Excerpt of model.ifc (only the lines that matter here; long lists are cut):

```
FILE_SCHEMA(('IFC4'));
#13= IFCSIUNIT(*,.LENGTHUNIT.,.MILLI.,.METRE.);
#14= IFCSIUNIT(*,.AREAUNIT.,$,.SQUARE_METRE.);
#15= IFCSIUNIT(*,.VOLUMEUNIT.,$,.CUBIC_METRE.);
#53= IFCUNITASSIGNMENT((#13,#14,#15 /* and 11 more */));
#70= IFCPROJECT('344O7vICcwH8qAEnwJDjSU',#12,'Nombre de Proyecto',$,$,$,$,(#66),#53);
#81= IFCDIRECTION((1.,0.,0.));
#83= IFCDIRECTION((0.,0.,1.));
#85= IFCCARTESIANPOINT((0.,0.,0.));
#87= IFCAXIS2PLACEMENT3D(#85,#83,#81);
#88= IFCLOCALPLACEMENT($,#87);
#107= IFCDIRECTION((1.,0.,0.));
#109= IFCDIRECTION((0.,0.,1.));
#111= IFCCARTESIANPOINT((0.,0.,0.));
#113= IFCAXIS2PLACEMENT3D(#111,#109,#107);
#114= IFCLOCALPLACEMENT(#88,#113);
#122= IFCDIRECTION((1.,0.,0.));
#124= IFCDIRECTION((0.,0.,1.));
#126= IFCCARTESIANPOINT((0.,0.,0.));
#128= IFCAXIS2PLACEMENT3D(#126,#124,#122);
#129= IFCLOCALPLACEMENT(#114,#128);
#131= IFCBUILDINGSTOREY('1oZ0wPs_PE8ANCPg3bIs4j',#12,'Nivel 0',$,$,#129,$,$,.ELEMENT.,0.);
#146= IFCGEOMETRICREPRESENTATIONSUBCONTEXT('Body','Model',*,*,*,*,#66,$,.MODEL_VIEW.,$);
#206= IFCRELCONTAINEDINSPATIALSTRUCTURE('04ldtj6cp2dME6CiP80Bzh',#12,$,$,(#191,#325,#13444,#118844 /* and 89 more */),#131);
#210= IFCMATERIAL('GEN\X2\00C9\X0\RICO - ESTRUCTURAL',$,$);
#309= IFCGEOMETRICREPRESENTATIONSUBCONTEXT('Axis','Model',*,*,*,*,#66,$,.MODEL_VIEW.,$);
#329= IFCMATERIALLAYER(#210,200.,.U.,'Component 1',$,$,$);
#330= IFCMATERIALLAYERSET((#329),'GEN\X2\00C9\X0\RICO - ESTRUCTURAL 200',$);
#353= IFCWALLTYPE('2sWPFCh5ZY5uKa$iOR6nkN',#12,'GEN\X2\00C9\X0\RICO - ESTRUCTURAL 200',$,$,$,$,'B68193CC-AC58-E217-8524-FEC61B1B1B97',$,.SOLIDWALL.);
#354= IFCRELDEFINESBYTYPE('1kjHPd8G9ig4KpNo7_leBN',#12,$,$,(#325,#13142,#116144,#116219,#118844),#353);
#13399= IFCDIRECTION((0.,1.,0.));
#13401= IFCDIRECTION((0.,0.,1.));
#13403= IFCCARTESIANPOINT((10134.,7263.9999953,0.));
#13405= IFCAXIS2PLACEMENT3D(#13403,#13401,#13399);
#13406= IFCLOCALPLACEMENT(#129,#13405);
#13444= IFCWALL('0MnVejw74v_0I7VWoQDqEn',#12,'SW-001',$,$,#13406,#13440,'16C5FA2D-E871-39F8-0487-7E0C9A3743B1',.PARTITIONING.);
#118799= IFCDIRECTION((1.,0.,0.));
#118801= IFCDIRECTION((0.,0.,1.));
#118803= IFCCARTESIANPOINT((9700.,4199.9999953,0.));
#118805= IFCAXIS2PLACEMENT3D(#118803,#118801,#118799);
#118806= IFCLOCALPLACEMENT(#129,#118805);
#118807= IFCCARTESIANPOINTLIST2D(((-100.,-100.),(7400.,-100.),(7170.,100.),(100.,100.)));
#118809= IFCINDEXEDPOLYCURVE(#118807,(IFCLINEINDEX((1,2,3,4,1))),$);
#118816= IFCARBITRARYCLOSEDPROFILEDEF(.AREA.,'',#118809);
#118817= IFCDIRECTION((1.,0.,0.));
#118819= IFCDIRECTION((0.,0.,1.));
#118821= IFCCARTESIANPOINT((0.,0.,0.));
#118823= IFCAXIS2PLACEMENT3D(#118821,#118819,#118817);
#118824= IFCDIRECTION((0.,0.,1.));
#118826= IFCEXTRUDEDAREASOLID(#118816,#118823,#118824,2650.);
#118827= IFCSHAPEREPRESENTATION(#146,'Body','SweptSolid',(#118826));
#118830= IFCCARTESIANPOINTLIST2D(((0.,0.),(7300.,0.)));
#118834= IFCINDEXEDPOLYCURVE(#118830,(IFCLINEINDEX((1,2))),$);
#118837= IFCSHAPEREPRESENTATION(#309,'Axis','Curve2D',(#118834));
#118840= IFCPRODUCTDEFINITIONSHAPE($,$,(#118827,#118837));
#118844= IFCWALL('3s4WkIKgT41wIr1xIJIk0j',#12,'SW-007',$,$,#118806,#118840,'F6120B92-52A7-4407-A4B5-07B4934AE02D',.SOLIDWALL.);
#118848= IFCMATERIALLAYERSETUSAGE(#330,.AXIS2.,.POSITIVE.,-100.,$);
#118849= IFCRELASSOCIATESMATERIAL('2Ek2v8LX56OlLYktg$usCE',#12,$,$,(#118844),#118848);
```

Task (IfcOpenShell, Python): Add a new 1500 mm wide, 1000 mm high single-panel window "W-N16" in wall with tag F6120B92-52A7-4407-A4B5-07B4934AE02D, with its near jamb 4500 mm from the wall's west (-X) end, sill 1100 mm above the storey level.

```python
import numpy as np
import ifcopenshell
import ifcopenshell.api.feature
import ifcopenshell.api.geometry
import ifcopenshell.api.root
import ifcopenshell.api.spatial
import ifcopenshell.geom
import ifcopenshell.util.element
import ifcopenshell.util.placement
import ifcopenshell.util.representation
import ifcopenshell.util.shape
import ifcopenshell.util.unit

model = ifcopenshell.open("model.ifc")
unit_scale = ifcopenshell.util.unit.calculate_unit_scale(model)
settings = ifcopenshell.geom.settings()


def volume(element):
    """Net volume in cubic metres, openings subtracted."""
    shape = ifcopenshell.geom.create_shape(settings, element)
    return ifcopenshell.util.shape.get_volume(shape.geometry)


wall = model.by_guid("3s4WkIKgT41wIr1xIJIk0j")
storey = ifcopenshell.util.element.get_container(wall, ifc_class="IfcBuildingStorey")
context = ifcopenshell.util.representation.get_context(model, "Model", "Body", "MODEL_VIEW")
before = volume(wall)

width, height, from_end, sill = 1.5, 1, 4.5, 1.1  # metres

# The wall runs along its own X axis, and the end named is its -X end.
wall_shape = ifcopenshell.geom.create_shape(settings, wall)
x, y, z = ifcopenshell.util.shape.get_vertices(wall_shape.geometry).T
start = x.min() + from_end
face, thickness = float(y.min()), float(y.max() - y.min())
wall_matrix = ifcopenshell.util.placement.get_local_placement(wall.ObjectPlacement)
level = ifcopenshell.util.placement.get_local_placement(storey.ObjectPlacement)[2, 3]


def in_wall(x, y):
    """Placement at x, y metres in the wall's axes, at sill height."""
    matrix = wall_matrix.copy()
    matrix[:, 3] = wall_matrix @ np.array([x / unit_scale, y / unit_scale, 0.0, 1.0])
    matrix[2, 3] = level + sill / unit_scale
    return matrix


# Opening: a box that overshoots both wall faces by 50 mm.
opening = ifcopenshell.api.root.create_entity(model, ifc_class="IfcOpeningElement", predefined_type="OPENING")
box = ifcopenshell.api.geometry.add_wall_representation(
    model, context=context, length=width, height=height, thickness=thickness + 0.1
)
ifcopenshell.api.geometry.assign_representation(model, product=opening, representation=box)
ifcopenshell.api.geometry.edit_object_placement(model, product=opening, matrix=in_wall(start, face - 0.05), is_si=False)
ifcopenshell.api.feature.add_feature(model, feature=opening, element=wall)

window = ifcopenshell.api.root.create_entity(model, ifc_class="IfcWindow", name="W-N16", predefined_type="WINDOW")
window.OverallWidth, window.OverallHeight = width / unit_scale, height / unit_scale
window.PartitioningType = "SINGLE_PANEL"
body = ifcopenshell.api.geometry.add_window_representation(
    model,
    context=context,
    overall_width=window.OverallWidth,
    overall_height=window.OverallHeight,
    partition_type="SINGLE_PANEL",
)
ifcopenshell.api.geometry.assign_representation(model, product=window, representation=body)
ifcopenshell.api.spatial.assign_container(model, products=[window], relating_structure=storey)
ifcopenshell.api.feature.add_filling(model, opening=opening, element=window)

# Centre the window in the wall's thickness.
ifcopenshell.api.geometry.edit_object_placement(model, product=window, matrix=in_wall(start, face), is_si=False)
window_shape = ifcopenshell.geom.create_shape(settings, window)
depth = ifcopenshell.util.shape.get_vertices(window_shape.geometry)[:, 1]
offset = face + thickness / 2 - (depth.min() + depth.max()) / 2
ifcopenshell.api.geometry.edit_object_placement(model, product=window, matrix=in_wall(start, offset), is_si=False)

after = volume(wall)

print(f"wall volume {before:.3f} -> {after:.3f} m3")

model.write("model_rev.ifc")
```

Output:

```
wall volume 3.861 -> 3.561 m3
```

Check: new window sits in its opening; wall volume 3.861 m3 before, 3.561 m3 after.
